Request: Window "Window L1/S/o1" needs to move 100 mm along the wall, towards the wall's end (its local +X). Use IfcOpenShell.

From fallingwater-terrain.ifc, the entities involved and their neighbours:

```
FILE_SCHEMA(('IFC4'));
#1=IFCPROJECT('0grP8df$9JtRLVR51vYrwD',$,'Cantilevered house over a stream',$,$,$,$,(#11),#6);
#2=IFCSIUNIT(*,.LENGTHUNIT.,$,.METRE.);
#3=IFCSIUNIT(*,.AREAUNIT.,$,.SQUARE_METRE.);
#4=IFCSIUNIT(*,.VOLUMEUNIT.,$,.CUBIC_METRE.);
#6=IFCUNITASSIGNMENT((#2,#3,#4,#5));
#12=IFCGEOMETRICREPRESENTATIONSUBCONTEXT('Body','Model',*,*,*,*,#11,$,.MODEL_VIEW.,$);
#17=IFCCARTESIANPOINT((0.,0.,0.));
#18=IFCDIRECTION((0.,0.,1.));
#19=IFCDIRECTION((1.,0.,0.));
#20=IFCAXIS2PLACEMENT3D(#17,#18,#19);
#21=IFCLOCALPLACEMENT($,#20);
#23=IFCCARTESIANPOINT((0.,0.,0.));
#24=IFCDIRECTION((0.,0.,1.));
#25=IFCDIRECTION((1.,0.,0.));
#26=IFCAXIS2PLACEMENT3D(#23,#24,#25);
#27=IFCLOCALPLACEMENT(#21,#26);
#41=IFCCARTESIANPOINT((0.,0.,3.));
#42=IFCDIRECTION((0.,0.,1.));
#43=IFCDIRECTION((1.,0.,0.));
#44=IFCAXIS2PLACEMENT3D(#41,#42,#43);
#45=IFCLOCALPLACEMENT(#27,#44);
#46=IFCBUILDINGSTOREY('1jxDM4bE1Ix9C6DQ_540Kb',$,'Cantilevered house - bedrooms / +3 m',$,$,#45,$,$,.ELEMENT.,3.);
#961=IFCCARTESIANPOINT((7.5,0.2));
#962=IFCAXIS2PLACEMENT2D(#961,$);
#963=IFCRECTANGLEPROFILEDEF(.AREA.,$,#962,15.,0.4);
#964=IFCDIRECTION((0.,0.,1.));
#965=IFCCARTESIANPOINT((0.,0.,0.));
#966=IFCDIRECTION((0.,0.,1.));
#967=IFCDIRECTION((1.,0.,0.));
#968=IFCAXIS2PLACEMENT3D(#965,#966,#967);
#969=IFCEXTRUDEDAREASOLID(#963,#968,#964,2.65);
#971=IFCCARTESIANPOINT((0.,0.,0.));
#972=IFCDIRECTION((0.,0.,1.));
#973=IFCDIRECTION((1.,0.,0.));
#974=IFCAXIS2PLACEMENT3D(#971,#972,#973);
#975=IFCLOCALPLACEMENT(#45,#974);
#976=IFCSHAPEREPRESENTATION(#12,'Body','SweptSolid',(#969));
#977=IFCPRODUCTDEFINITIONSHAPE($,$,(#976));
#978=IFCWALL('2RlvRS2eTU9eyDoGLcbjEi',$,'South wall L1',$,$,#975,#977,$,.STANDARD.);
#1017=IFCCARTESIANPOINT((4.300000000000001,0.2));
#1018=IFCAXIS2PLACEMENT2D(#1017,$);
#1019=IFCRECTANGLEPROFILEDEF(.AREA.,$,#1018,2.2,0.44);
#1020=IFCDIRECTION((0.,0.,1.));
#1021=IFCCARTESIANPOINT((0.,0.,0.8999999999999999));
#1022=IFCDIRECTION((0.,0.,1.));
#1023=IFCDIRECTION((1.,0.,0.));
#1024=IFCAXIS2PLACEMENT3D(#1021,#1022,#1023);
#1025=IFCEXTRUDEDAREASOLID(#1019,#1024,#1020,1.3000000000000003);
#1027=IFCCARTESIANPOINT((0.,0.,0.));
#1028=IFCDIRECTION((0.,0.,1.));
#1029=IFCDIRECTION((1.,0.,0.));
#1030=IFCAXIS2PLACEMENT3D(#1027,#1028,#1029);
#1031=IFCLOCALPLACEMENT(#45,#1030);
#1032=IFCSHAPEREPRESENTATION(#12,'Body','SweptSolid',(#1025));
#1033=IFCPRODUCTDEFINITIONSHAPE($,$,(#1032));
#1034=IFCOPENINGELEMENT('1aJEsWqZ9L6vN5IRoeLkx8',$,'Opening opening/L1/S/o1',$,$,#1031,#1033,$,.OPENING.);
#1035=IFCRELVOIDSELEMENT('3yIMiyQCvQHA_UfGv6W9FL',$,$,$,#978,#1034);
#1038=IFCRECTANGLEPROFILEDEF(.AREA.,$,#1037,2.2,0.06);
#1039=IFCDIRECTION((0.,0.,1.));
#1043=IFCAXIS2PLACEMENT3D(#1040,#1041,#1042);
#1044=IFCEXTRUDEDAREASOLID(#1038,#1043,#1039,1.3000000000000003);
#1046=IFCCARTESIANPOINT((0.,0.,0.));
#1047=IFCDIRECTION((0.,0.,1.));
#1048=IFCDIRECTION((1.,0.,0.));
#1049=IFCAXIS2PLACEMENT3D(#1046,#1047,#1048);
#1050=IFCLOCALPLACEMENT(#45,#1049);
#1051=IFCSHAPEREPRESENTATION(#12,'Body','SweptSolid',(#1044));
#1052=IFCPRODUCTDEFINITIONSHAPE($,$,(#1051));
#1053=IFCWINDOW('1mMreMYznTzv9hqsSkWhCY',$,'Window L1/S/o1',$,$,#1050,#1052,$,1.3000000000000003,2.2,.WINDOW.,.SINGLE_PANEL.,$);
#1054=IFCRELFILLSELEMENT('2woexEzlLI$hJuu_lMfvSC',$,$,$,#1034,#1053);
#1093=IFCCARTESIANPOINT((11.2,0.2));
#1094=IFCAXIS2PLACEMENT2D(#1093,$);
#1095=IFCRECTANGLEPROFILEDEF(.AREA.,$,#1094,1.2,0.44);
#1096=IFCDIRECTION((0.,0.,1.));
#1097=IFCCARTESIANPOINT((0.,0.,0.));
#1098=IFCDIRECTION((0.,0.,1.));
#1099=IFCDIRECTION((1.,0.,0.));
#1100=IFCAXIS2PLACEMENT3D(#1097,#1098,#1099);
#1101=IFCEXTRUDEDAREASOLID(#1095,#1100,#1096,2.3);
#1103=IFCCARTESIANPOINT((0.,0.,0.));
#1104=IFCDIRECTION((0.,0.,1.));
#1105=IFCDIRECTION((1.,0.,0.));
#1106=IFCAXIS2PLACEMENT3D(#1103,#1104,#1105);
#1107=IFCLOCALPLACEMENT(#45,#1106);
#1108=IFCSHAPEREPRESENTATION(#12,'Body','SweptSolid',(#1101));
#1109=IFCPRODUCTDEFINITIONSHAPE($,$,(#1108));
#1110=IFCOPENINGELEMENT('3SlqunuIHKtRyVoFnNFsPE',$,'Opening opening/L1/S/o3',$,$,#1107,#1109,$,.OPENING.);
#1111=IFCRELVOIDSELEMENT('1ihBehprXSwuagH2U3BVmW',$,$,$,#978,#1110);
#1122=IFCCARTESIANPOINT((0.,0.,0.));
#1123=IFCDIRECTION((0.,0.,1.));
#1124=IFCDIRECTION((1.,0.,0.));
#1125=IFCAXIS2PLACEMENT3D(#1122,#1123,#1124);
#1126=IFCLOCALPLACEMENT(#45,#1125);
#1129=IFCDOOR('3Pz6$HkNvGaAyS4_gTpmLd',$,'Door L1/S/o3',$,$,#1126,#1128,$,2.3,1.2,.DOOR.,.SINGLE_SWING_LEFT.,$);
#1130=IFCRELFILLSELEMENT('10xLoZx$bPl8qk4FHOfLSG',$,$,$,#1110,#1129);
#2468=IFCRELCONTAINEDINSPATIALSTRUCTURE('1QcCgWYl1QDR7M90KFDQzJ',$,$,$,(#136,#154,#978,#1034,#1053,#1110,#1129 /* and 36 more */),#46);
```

```python
import ifcopenshell
import ifcopenshell.api.geometry
import ifcopenshell.util.placement
import ifcopenshell.util.unit

model = ifcopenshell.open("fallingwater-terrain.ifc")
unit_scale = ifcopenshell.util.unit.calculate_unit_scale(model)

window = model.by_guid("1mMreMYznTzv9hqsSkWhCY")
opening = window.FillsVoids[0].RelatingOpeningElement
wall = opening.VoidsElements[0].RelatingBuildingElement

wall_matrix = ifcopenshell.util.placement.get_local_placement(wall.ObjectPlacement)
shift = wall_matrix[:3, 0] * 0.1 / unit_scale
before = ifcopenshell.util.placement.get_local_placement(window.ObjectPlacement)[:3, 3].copy()

# The window is not placed relative to its opening, so move both.
for product in (opening, window):
    matrix = ifcopenshell.util.placement.get_local_placement(product.ObjectPlacement)
    matrix[:3, 3] += shift
    ifcopenshell.api.geometry.edit_object_placement(model, product=product, matrix=matrix, is_si=False)

after = ifcopenshell.util.placement.get_local_placement(window.ObjectPlacement)[:3, 3]
print("window moved by", (after - before).round(3) + 0.0)

model.write("fallingwater-terrain_edited.ifc")
```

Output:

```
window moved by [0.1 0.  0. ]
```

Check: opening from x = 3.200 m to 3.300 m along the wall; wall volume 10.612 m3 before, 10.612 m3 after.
